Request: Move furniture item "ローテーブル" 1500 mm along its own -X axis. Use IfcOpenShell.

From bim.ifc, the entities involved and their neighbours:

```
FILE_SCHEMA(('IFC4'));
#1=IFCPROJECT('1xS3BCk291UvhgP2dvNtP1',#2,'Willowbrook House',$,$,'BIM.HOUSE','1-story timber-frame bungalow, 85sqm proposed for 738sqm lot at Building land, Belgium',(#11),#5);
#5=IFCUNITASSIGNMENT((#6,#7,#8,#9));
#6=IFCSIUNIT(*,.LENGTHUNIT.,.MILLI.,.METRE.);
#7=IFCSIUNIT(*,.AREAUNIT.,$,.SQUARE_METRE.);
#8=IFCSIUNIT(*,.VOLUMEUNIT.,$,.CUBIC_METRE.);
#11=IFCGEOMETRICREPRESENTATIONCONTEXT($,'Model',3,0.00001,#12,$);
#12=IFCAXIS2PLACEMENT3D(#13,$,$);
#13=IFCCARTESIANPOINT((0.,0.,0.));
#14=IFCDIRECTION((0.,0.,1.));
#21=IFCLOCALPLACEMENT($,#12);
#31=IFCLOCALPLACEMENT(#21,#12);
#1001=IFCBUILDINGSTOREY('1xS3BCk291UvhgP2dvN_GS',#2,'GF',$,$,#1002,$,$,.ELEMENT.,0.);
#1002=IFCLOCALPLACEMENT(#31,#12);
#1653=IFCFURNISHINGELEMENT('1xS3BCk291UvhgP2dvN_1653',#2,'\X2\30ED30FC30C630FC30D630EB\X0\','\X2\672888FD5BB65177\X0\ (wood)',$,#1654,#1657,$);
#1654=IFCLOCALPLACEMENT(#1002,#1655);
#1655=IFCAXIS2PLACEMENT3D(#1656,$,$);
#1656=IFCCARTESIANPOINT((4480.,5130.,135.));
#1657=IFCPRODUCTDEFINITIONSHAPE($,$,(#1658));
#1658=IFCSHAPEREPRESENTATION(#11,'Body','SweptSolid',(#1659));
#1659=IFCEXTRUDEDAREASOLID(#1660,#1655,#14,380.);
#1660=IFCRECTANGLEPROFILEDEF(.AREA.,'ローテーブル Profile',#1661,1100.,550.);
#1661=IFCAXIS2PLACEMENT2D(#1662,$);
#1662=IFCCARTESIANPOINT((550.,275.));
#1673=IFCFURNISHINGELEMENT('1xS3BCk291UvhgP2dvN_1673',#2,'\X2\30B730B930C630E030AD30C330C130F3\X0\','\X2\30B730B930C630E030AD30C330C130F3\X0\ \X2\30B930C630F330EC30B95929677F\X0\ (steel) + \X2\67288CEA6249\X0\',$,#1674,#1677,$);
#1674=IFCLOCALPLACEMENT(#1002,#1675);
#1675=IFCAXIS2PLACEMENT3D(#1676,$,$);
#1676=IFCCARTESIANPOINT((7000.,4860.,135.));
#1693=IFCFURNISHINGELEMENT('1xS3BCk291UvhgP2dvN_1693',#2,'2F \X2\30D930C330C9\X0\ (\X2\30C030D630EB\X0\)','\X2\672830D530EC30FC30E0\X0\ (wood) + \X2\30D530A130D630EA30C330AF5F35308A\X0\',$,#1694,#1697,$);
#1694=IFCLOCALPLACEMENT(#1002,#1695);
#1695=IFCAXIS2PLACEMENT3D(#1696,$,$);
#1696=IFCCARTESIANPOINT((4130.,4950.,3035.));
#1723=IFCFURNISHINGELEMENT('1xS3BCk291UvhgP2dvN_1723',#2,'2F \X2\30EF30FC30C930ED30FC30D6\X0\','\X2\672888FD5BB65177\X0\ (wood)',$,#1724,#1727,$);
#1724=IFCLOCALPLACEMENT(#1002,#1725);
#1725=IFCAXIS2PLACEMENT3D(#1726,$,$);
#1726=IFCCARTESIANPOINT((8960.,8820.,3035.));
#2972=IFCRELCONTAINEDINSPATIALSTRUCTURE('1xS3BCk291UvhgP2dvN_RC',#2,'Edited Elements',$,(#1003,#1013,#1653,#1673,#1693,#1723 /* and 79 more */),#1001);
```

```python
import ifcopenshell
import ifcopenshell.api.geometry
import ifcopenshell.util.placement
import ifcopenshell.util.unit

model = ifcopenshell.open("bim.ifc")
unit_scale = ifcopenshell.util.unit.calculate_unit_scale(model)

item = model.by_id(1653)
matrix = ifcopenshell.util.placement.get_local_placement(item.ObjectPlacement)
matrix[:3, 3] -= matrix[:3, 0] * 1.5 / unit_scale
ifcopenshell.api.geometry.edit_object_placement(model, product=item, matrix=matrix, is_si=False)

print(ifcopenshell.util.placement.get_local_placement(item.ObjectPlacement).round(3) + 0.0)

model.write("bim_rev.ifc")
```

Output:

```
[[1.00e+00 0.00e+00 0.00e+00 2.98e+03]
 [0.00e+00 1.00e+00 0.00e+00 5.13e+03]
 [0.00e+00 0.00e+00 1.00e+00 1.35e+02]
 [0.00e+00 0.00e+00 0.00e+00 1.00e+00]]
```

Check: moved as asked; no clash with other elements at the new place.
